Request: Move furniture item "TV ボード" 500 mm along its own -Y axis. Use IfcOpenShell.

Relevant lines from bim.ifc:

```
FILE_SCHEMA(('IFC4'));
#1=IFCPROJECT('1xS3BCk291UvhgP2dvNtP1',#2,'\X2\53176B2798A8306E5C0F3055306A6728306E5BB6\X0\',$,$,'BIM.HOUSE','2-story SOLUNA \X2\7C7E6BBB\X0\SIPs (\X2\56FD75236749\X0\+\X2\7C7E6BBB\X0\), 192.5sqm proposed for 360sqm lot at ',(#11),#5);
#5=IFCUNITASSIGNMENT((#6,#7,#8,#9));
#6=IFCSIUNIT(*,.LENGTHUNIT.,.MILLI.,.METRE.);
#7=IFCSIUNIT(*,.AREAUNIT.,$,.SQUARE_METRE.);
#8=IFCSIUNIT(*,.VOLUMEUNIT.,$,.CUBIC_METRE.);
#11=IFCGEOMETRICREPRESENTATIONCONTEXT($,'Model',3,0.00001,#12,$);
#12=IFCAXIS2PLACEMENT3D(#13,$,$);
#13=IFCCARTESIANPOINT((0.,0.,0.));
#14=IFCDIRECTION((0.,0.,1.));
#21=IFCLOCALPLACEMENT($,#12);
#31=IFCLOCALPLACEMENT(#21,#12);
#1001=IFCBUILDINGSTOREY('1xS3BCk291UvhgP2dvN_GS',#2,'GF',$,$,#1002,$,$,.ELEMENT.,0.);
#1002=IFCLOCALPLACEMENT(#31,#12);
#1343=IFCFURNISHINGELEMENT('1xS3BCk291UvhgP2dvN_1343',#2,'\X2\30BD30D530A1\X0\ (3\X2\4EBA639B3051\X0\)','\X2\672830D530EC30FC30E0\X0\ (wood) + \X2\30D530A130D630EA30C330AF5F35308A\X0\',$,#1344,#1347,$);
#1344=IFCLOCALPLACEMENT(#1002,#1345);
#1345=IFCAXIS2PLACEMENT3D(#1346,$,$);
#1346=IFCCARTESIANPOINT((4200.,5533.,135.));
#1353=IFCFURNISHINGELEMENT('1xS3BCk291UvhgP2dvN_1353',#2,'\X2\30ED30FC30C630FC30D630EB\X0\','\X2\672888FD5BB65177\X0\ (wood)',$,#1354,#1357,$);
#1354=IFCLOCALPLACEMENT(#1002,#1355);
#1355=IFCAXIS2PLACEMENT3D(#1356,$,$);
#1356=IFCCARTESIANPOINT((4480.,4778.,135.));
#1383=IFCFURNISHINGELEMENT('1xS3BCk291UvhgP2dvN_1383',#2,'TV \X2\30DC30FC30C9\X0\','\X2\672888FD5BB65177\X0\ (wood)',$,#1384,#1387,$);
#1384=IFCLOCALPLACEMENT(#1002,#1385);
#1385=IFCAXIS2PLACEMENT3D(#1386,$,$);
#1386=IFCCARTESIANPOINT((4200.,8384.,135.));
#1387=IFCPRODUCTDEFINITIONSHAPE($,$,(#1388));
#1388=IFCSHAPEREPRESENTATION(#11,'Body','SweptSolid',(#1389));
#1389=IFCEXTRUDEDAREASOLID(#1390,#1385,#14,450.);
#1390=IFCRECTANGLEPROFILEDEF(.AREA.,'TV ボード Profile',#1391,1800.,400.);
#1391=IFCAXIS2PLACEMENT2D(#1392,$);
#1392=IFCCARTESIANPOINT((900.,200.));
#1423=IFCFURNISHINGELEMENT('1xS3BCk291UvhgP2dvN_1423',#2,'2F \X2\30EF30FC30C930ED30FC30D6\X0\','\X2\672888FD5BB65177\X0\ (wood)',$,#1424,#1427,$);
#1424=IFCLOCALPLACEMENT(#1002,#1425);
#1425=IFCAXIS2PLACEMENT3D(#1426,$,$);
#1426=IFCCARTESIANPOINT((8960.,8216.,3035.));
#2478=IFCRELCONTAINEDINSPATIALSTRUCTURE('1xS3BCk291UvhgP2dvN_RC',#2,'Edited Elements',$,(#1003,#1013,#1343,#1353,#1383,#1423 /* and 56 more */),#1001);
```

```python
import ifcopenshell
import ifcopenshell.api.geometry
import ifcopenshell.util.placement
import ifcopenshell.util.unit

model = ifcopenshell.open("bim.ifc")
unit_scale = ifcopenshell.util.unit.calculate_unit_scale(model)

item = model.by_guid("1xS3BCk291UvhgP2dvN_1383")
matrix = ifcopenshell.util.placement.get_local_placement(item.ObjectPlacement)
matrix[:3, 3] -= matrix[:3, 1] * 0.5 / unit_scale
ifcopenshell.api.geometry.edit_object_placement(model, product=item, matrix=matrix, is_si=False)

print(ifcopenshell.util.placement.get_local_placement(item.ObjectPlacement).round(3) + 0.0)

model.write("bim_edited.ifc")
```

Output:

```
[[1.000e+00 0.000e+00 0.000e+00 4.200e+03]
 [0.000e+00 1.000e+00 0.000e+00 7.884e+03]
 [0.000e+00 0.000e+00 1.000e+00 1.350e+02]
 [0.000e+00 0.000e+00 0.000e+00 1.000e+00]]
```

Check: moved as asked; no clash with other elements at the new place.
